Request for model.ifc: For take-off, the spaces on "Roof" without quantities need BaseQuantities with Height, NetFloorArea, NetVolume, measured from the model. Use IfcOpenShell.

First a look at what the model holds.

```python
import ifcopenshell
import ifcopenshell.util.element
import ifcopenshell.util.unit

model = ifcopenshell.open("model.ifc")
print(model.schema)
for unit_type in ("LENGTHUNIT", "AREAUNIT", "VOLUMEUNIT"):
    print(unit_type, ifcopenshell.util.unit.calculate_unit_scale(model, unit_type))
storey = next(s for s in model.by_type("IfcBuildingStorey") if s.Name == "Roof")
spaces = [e for e in ifcopenshell.util.element.get_decomposition(storey) if e.is_a("IfcSpace")]
for e in sorted(spaces, key=lambda e: e.id()):
    print(e.id(), e.is_a(), e.Name, list(ifcopenshell.util.element.get_psets(e, qtos_only=True)), sep=" | ")
```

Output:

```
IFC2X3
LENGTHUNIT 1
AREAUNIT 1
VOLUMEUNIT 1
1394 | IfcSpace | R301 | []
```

```python
import ifcopenshell
import ifcopenshell.api.pset
import ifcopenshell.geom
import ifcopenshell.util.element
import ifcopenshell.util.shape
import ifcopenshell.util.unit

model = ifcopenshell.open("model.ifc")
unit_scale = ifcopenshell.util.unit.calculate_unit_scale(model)
area_scale = ifcopenshell.util.unit.calculate_unit_scale(model, "AREAUNIT")
volume_scale = ifcopenshell.util.unit.calculate_unit_scale(model, "VOLUMEUNIT")
settings = ifcopenshell.geom.settings()

storey = next(s for s in model.by_type("IfcBuildingStorey") if s.Name == "Roof")
spaces = [e for e in ifcopenshell.util.element.get_decomposition(storey) if e.is_a("IfcSpace")]

for e in sorted(spaces, key=lambda e: e.id()):
    if ifcopenshell.util.element.get_psets(e, qtos_only=True, should_inherit=False):
        continue
    # Geometry comes back in metres, in the element's own axes.
    shape = ifcopenshell.geom.create_shape(settings, e)
    values = {
        "Height": ifcopenshell.util.shape.get_z(shape.geometry) / unit_scale,
        "NetFloorArea": ifcopenshell.util.shape.get_footprint_area(shape.geometry) / area_scale,
        "NetVolume": ifcopenshell.util.shape.get_volume(shape.geometry) / volume_scale,
    }
    qto = ifcopenshell.api.pset.add_qto(model, product=e, name="BaseQuantities")
    ifcopenshell.api.pset.edit_qto(model, qto=qto, properties=values)
    print(e.id(), {k: round(v, 3) for k, v in values.items()})

model.write("model_edited.ifc")
```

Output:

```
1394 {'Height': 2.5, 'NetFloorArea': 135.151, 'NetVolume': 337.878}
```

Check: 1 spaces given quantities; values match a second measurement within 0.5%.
